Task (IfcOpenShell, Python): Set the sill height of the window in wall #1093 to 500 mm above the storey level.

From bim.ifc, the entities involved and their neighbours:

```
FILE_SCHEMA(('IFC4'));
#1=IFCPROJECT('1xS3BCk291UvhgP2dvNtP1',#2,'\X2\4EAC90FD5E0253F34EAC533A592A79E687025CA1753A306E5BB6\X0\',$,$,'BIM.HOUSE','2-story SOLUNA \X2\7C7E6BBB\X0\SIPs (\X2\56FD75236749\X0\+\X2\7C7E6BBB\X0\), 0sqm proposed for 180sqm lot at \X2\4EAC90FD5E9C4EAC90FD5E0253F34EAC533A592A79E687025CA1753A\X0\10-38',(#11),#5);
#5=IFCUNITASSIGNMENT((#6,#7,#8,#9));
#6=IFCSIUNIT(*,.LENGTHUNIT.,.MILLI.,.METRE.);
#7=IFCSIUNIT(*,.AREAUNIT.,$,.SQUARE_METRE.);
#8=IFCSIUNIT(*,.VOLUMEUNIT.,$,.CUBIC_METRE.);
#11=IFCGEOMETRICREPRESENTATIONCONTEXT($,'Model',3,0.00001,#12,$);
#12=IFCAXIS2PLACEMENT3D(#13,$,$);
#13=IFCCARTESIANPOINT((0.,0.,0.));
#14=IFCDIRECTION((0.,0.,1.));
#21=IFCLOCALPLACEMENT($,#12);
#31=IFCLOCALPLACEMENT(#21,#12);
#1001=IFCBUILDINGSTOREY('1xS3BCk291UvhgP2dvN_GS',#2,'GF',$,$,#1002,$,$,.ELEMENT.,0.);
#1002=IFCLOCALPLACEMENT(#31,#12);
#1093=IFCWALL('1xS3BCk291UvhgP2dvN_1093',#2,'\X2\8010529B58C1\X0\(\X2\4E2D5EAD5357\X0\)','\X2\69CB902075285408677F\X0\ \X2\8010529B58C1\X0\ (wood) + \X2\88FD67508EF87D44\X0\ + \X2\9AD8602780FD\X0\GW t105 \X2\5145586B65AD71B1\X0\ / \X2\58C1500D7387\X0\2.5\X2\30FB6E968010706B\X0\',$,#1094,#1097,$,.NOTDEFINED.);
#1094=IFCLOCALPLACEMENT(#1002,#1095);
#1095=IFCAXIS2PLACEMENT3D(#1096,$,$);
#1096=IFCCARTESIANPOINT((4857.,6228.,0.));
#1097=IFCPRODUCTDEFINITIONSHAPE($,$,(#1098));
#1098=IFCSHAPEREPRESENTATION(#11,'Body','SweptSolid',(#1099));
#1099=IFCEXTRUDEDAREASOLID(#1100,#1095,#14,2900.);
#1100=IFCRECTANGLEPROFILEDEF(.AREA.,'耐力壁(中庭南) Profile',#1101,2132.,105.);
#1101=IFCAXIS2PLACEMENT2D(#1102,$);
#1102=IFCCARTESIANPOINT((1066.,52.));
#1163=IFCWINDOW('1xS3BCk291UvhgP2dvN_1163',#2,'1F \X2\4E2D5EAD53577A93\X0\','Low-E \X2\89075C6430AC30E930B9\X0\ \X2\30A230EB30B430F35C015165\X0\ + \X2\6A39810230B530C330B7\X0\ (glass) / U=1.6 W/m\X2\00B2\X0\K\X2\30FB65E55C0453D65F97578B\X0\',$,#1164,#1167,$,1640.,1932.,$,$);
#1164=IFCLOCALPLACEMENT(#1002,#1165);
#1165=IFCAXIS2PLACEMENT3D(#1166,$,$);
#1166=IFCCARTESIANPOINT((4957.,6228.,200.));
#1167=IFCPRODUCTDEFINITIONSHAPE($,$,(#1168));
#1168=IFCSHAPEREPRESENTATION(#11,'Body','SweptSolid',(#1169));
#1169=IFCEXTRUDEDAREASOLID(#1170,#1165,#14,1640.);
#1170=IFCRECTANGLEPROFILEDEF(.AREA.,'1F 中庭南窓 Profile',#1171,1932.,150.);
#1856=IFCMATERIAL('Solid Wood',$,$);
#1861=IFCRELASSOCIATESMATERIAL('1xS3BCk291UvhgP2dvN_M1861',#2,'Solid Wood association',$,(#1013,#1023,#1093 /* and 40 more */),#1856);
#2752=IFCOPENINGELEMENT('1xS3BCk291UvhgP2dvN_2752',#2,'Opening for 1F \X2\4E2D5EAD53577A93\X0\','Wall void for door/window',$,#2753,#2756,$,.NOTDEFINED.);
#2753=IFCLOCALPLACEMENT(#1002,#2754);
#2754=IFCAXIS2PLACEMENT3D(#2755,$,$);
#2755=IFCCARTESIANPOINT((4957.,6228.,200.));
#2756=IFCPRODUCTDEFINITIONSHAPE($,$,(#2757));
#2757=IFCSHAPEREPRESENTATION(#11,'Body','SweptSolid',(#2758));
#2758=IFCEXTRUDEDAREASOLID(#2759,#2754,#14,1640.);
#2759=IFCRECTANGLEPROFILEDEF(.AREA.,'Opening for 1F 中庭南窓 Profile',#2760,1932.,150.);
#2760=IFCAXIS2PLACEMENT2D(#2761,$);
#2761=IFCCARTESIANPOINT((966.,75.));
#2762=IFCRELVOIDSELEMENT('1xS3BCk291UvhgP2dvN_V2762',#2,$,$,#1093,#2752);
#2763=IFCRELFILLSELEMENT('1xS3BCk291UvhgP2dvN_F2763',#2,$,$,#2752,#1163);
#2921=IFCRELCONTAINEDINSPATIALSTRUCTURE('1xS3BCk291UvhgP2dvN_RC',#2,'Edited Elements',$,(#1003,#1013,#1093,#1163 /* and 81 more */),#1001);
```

```python
import numpy as np
import ifcopenshell
import ifcopenshell.api.geometry
import ifcopenshell.geom
import ifcopenshell.util.element
import ifcopenshell.util.placement
import ifcopenshell.util.shape
import ifcopenshell.util.unit

model = ifcopenshell.open("bim.ifc")
unit_scale = ifcopenshell.util.unit.calculate_unit_scale(model)

window = model.by_id(1163)
opening = window.FillsVoids[0].RelatingOpeningElement
storey = ifcopenshell.util.element.get_container(window, ifc_class="IfcBuildingStorey")
level = ifcopenshell.util.placement.get_local_placement(storey.ObjectPlacement)[2, 3]

# The opening's origin need not be at the sill, so measure its lowest point.
shape = ifcopenshell.geom.create_shape(ifcopenshell.geom.settings(), opening)
bottom = ifcopenshell.util.shape.get_shape_bottom_elevation(shape, shape.geometry) / unit_scale
dz = level + 500.0 - bottom

shift = np.array([0.0, 0.0, dz])
# The window is not placed relative to its opening, so move both.
for product in (opening, window):
    matrix = ifcopenshell.util.placement.get_local_placement(product.ObjectPlacement)
    matrix[:3, 3] += shift
    ifcopenshell.api.geometry.edit_object_placement(model, product=product, matrix=matrix, is_si=False)

print(f"moved by {dz * unit_scale:+.3f} m")

model.write("bim_rev.ifc")
```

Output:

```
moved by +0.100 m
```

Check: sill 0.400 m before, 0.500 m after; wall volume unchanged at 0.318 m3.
